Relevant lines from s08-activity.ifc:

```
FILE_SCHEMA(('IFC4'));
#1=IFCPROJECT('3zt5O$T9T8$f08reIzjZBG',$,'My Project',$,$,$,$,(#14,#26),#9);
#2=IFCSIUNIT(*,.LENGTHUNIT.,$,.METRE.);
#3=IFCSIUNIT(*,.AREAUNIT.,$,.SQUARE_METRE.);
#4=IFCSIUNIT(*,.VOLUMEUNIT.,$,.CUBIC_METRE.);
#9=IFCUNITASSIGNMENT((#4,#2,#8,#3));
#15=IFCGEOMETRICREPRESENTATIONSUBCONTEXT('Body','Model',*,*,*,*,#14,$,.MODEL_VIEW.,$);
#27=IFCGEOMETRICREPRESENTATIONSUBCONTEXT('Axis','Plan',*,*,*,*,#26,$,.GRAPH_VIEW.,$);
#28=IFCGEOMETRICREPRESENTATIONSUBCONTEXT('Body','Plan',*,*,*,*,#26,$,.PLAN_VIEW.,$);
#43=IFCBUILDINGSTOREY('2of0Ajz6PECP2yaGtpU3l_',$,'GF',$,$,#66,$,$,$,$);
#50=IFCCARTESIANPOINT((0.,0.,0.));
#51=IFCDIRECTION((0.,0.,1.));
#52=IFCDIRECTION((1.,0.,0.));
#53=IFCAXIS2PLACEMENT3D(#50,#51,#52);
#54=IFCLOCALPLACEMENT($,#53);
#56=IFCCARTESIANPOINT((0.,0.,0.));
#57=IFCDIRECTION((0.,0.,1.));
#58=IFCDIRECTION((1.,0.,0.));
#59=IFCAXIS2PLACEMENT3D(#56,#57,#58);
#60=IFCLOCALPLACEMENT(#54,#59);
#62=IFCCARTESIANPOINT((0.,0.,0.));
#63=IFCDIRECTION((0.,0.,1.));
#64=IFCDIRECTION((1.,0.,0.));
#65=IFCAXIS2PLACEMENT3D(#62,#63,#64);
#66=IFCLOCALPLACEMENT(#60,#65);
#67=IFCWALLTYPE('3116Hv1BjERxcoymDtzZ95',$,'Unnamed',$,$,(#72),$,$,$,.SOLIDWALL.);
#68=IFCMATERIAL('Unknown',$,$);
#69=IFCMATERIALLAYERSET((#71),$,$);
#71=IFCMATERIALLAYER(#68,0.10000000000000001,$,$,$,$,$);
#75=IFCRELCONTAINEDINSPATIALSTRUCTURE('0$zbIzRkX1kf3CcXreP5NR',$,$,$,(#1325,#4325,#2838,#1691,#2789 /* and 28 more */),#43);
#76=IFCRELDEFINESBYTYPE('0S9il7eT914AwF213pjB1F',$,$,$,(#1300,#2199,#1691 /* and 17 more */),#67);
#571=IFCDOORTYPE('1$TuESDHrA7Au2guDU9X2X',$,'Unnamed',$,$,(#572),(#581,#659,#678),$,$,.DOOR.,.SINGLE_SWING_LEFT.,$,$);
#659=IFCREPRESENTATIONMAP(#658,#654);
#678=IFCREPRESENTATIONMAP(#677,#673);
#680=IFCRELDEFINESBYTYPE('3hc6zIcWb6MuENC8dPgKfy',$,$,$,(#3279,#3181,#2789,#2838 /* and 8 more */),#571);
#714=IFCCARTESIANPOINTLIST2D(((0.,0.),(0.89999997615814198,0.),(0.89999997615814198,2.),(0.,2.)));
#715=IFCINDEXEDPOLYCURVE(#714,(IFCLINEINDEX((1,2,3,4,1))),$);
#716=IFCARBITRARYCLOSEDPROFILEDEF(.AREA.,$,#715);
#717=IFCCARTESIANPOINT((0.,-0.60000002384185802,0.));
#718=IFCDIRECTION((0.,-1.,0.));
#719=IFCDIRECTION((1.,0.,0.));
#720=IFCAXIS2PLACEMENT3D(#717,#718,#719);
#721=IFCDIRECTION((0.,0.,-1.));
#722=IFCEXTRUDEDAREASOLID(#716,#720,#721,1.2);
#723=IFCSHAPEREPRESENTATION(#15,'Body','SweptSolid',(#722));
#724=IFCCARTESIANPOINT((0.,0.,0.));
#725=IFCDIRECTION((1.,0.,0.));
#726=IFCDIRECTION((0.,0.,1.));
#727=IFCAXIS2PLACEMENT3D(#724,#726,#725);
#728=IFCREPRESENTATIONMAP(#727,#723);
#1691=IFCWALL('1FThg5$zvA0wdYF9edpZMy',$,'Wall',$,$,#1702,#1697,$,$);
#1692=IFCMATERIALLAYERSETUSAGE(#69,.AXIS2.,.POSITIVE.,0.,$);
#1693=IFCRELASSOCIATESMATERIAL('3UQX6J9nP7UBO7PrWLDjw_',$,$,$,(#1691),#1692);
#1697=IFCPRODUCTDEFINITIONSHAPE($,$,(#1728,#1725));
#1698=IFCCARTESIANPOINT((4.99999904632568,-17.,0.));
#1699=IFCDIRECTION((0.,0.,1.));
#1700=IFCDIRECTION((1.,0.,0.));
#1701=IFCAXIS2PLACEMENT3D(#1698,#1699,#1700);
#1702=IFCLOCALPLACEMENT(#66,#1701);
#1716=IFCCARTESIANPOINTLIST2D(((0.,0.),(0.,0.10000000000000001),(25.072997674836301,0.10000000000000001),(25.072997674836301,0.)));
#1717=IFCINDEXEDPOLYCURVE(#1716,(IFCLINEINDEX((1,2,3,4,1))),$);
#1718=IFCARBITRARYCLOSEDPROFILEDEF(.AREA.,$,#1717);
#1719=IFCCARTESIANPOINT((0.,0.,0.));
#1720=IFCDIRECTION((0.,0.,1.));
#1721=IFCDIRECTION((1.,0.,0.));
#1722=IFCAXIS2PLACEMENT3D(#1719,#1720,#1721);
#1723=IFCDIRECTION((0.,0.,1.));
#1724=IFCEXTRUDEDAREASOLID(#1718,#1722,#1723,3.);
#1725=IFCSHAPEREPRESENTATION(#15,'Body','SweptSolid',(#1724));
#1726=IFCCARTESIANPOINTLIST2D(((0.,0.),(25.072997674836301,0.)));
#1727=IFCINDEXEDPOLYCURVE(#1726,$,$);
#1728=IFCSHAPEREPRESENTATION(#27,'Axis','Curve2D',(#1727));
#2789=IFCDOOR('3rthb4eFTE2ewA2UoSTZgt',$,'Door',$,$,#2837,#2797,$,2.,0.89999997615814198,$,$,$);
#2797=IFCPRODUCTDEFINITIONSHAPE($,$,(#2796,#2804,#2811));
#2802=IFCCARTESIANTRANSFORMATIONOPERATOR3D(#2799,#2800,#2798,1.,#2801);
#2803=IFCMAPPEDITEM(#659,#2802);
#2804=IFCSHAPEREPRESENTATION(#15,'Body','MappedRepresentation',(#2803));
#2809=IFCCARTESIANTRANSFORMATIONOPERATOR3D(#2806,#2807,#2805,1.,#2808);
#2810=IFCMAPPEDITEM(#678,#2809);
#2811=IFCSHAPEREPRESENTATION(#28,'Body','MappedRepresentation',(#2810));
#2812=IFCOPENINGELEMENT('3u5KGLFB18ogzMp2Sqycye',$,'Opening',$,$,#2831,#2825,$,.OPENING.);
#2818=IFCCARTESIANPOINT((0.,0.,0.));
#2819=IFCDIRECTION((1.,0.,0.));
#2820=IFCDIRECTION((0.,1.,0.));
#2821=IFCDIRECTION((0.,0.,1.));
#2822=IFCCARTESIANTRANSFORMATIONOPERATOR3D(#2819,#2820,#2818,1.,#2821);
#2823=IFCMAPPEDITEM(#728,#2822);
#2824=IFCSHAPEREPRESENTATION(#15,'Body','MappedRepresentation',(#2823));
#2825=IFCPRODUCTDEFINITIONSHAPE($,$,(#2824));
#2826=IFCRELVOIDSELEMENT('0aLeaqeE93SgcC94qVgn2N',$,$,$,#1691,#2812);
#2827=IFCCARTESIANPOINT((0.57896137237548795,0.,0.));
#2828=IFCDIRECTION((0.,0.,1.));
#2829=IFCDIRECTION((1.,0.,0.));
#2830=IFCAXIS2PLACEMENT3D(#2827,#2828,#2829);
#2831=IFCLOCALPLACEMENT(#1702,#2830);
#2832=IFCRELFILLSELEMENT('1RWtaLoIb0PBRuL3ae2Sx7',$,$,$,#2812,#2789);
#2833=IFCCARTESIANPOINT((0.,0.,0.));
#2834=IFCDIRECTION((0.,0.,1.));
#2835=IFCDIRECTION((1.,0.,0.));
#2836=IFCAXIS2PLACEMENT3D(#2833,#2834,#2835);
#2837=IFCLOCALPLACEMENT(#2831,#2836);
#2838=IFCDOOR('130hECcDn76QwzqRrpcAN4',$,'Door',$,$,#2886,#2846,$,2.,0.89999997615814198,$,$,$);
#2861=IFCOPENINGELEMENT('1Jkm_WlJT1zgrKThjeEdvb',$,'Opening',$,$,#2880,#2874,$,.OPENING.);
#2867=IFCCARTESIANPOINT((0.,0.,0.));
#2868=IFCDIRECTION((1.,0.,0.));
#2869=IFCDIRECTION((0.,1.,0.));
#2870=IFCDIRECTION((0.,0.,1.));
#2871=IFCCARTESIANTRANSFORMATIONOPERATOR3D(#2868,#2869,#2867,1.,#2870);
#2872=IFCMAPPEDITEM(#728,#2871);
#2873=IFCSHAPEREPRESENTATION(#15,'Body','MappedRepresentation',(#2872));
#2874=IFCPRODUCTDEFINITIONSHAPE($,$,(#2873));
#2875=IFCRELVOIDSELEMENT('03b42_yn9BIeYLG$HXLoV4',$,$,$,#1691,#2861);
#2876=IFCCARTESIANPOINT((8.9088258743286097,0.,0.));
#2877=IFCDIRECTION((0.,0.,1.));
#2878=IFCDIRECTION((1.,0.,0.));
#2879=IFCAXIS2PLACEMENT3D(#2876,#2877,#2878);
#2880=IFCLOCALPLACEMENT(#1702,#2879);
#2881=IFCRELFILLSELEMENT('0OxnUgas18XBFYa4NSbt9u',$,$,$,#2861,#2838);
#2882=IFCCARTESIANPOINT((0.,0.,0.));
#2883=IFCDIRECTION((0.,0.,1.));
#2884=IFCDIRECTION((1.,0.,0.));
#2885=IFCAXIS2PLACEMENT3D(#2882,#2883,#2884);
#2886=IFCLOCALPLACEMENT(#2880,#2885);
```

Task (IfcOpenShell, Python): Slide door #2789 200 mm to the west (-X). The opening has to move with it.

```python
import ifcopenshell
import ifcopenshell.api.geometry
import ifcopenshell.util.placement

model = ifcopenshell.open("s08-activity.ifc")

door = model.by_guid("3rthb4eFTE2ewA2UoSTZgt")
opening = door.FillsVoids[0].RelatingOpeningElement
wall = opening.VoidsElements[0].RelatingBuildingElement

wall_matrix = ifcopenshell.util.placement.get_local_placement(wall.ObjectPlacement)
shift = wall_matrix[:3, 0] * -0.2
before = ifcopenshell.util.placement.get_local_placement(door.ObjectPlacement)[:3, 3].copy()

# The door is placed relative to its opening, so it follows when the opening moves.
matrix = ifcopenshell.util.placement.get_local_placement(opening.ObjectPlacement)
matrix[:3, 3] += shift
ifcopenshell.api.geometry.edit_object_placement(
    model, product=opening, matrix=matrix, is_si=False, should_transform_children=True
)

after = ifcopenshell.util.placement.get_local_placement(door.ObjectPlacement)[:3, 3]
print("door moved by", (after - before).round(3) + 0.0)

model.write("s08-activity_edited.ifc")
```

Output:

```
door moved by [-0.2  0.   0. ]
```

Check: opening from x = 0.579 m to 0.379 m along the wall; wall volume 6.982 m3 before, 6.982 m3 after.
